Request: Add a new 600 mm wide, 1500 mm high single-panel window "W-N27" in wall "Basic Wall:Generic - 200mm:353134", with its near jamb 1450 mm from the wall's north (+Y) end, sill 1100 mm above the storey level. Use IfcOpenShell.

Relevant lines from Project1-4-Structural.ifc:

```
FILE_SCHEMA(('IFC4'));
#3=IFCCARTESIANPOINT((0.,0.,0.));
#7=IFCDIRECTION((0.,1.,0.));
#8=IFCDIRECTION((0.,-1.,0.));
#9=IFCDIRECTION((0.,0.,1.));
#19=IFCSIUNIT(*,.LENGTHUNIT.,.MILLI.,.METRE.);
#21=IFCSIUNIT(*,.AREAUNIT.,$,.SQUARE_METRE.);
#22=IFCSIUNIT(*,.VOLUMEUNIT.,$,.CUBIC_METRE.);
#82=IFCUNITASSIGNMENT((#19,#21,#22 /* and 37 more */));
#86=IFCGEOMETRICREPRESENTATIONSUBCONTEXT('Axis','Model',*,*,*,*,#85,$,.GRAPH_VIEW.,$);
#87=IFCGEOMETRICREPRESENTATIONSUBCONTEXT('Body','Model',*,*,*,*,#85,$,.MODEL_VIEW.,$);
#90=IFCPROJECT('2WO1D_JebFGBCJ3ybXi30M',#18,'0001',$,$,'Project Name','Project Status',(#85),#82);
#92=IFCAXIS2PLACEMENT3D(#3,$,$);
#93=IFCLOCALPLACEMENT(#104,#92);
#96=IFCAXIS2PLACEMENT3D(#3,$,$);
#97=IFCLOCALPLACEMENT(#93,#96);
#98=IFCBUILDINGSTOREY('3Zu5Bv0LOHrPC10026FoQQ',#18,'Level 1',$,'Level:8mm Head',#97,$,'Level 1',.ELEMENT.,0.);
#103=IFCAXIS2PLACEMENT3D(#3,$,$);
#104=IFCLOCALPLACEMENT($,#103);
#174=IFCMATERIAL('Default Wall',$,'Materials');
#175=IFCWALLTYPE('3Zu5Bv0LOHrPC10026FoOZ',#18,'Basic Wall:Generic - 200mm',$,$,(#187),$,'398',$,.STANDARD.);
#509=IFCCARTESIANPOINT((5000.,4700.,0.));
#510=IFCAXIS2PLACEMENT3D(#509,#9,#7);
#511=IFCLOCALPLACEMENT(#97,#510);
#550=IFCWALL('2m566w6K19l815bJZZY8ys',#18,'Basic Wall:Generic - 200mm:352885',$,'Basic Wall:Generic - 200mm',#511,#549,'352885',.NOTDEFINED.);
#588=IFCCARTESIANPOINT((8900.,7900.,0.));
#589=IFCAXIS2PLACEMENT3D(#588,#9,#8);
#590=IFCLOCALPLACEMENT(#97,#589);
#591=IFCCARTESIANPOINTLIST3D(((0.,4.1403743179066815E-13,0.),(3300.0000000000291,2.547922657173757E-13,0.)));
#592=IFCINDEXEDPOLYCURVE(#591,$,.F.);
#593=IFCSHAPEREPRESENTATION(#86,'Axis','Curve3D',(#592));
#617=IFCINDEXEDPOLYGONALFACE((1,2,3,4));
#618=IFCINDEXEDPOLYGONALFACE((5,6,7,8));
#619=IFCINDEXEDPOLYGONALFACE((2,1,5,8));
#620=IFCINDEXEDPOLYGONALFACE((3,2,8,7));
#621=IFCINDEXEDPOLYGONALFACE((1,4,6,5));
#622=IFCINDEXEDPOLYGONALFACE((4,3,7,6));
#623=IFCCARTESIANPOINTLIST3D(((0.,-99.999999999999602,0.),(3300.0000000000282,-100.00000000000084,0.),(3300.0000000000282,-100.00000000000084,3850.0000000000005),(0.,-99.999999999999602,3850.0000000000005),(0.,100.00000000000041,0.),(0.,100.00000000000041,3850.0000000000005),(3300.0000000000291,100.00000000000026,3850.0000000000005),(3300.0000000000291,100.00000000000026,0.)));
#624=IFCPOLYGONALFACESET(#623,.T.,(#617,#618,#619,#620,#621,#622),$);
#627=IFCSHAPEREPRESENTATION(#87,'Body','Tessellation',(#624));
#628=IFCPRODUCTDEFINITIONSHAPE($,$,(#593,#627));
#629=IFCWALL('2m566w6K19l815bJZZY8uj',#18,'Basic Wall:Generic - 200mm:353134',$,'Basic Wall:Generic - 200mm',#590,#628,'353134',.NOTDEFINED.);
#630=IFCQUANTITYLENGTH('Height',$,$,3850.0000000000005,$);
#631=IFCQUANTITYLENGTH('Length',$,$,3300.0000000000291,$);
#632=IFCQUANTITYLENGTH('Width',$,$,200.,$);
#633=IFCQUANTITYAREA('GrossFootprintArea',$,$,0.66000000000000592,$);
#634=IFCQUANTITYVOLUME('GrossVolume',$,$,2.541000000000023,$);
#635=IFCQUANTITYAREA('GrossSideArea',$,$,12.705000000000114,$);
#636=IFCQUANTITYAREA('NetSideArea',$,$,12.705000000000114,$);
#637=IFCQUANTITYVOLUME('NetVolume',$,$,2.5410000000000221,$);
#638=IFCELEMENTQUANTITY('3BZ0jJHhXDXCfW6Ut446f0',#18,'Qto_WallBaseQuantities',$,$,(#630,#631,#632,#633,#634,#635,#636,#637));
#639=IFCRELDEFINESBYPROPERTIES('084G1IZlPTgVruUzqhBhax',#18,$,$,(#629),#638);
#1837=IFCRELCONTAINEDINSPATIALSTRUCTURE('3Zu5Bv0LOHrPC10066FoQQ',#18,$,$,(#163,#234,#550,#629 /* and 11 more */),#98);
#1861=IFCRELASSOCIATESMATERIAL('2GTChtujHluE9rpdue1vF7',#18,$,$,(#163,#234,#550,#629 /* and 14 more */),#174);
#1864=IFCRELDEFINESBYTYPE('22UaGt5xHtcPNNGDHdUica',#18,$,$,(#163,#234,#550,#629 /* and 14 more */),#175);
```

```python
import numpy as np
import ifcopenshell
import ifcopenshell.api.feature
import ifcopenshell.api.geometry
import ifcopenshell.api.pset
import ifcopenshell.api.root
import ifcopenshell.api.spatial
import ifcopenshell.geom
import ifcopenshell.util.element
import ifcopenshell.util.placement
import ifcopenshell.util.representation
import ifcopenshell.util.shape
import ifcopenshell.util.unit

model = ifcopenshell.open("Project1-4-Structural.ifc")
unit_scale = ifcopenshell.util.unit.calculate_unit_scale(model)
area_scale = ifcopenshell.util.unit.calculate_unit_scale(model, "AREAUNIT")
volume_scale = ifcopenshell.util.unit.calculate_unit_scale(model, "VOLUMEUNIT")
settings = ifcopenshell.geom.settings()


def volume(element):
    """Net volume in cubic metres, openings subtracted."""
    shape = ifcopenshell.geom.create_shape(settings, element)
    return ifcopenshell.util.shape.get_volume(shape.geometry)


wall = model.by_guid("2m566w6K19l815bJZZY8uj")
storey = ifcopenshell.util.element.get_container(wall, ifc_class="IfcBuildingStorey")
context = ifcopenshell.util.representation.get_context(model, "Model", "Body", "MODEL_VIEW")
before = volume(wall)

width, height, from_end, sill = 0.6, 1.5, 1.45, 1.1  # metres

# The wall runs along its own X axis, and the end named is its -X end.
wall_shape = ifcopenshell.geom.create_shape(settings, wall)
x, y, z = ifcopenshell.util.shape.get_vertices(wall_shape.geometry).T
start = x.min() + from_end
face, thickness = float(y.min()), float(y.max() - y.min())
wall_matrix = ifcopenshell.util.placement.get_local_placement(wall.ObjectPlacement)
level = ifcopenshell.util.placement.get_local_placement(storey.ObjectPlacement)[2, 3]


def in_wall(x, y):
    """Placement at x, y metres in the wall's axes, at sill height."""
    matrix = wall_matrix.copy()
    matrix[:, 3] = wall_matrix @ np.array([x / unit_scale, y / unit_scale, 0.0, 1.0])
    matrix[2, 3] = level + sill / unit_scale
    return matrix


# Opening: a box that overshoots both wall faces by 50 mm.
opening = ifcopenshell.api.root.create_entity(model, ifc_class="IfcOpeningElement", predefined_type="OPENING")
box = ifcopenshell.api.geometry.add_wall_representation(
    model, context=context, length=width, height=height, thickness=thickness + 0.1
)
ifcopenshell.api.geometry.assign_representation(model, product=opening, representation=box)
ifcopenshell.api.geometry.edit_object_placement(model, product=opening, matrix=in_wall(start, face - 0.05), is_si=False)
ifcopenshell.api.feature.add_feature(model, feature=opening, element=wall)

window = ifcopenshell.api.root.create_entity(model, ifc_class="IfcWindow", name="W-N27", predefined_type="WINDOW")
window.OverallWidth, window.OverallHeight = width / unit_scale, height / unit_scale
window.PartitioningType = "SINGLE_PANEL"
body = ifcopenshell.api.geometry.add_window_representation(
    model,
    context=context,
    overall_width=window.OverallWidth,
    overall_height=window.OverallHeight,
    partition_type="SINGLE_PANEL",
)
ifcopenshell.api.geometry.assign_representation(model, product=window, representation=body)
ifcopenshell.api.spatial.assign_container(model, products=[window], relating_structure=storey)
ifcopenshell.api.feature.add_filling(model, opening=opening, element=window)

# Centre the window in the wall's thickness.
ifcopenshell.api.geometry.edit_object_placement(model, product=window, matrix=in_wall(start, face), is_si=False)
window_shape = ifcopenshell.geom.create_shape(settings, window)
depth = ifcopenshell.util.shape.get_vertices(window_shape.geometry)[:, 1]
offset = face + thickness / 2 - (depth.min() + depth.max()) / 2
ifcopenshell.api.geometry.edit_object_placement(model, product=window, matrix=in_wall(start, offset), is_si=False)

after = volume(wall)

# Update the wall's stored quantities.
qto = model.by_id(ifcopenshell.util.element.get_pset(wall, "Qto_WallBaseQuantities", should_inherit=False)["id"])
ifcopenshell.api.pset.edit_qto(model, qto=qto, properties={
    "NetSideArea": after / thickness / area_scale,
    "NetVolume": after / volume_scale,
})

print(f"wall volume {before:.3f} -> {after:.3f} m3")

model.write("Project1-4-Structural_updated.ifc")
```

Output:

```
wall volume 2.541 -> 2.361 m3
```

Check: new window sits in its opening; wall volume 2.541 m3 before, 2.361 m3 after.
